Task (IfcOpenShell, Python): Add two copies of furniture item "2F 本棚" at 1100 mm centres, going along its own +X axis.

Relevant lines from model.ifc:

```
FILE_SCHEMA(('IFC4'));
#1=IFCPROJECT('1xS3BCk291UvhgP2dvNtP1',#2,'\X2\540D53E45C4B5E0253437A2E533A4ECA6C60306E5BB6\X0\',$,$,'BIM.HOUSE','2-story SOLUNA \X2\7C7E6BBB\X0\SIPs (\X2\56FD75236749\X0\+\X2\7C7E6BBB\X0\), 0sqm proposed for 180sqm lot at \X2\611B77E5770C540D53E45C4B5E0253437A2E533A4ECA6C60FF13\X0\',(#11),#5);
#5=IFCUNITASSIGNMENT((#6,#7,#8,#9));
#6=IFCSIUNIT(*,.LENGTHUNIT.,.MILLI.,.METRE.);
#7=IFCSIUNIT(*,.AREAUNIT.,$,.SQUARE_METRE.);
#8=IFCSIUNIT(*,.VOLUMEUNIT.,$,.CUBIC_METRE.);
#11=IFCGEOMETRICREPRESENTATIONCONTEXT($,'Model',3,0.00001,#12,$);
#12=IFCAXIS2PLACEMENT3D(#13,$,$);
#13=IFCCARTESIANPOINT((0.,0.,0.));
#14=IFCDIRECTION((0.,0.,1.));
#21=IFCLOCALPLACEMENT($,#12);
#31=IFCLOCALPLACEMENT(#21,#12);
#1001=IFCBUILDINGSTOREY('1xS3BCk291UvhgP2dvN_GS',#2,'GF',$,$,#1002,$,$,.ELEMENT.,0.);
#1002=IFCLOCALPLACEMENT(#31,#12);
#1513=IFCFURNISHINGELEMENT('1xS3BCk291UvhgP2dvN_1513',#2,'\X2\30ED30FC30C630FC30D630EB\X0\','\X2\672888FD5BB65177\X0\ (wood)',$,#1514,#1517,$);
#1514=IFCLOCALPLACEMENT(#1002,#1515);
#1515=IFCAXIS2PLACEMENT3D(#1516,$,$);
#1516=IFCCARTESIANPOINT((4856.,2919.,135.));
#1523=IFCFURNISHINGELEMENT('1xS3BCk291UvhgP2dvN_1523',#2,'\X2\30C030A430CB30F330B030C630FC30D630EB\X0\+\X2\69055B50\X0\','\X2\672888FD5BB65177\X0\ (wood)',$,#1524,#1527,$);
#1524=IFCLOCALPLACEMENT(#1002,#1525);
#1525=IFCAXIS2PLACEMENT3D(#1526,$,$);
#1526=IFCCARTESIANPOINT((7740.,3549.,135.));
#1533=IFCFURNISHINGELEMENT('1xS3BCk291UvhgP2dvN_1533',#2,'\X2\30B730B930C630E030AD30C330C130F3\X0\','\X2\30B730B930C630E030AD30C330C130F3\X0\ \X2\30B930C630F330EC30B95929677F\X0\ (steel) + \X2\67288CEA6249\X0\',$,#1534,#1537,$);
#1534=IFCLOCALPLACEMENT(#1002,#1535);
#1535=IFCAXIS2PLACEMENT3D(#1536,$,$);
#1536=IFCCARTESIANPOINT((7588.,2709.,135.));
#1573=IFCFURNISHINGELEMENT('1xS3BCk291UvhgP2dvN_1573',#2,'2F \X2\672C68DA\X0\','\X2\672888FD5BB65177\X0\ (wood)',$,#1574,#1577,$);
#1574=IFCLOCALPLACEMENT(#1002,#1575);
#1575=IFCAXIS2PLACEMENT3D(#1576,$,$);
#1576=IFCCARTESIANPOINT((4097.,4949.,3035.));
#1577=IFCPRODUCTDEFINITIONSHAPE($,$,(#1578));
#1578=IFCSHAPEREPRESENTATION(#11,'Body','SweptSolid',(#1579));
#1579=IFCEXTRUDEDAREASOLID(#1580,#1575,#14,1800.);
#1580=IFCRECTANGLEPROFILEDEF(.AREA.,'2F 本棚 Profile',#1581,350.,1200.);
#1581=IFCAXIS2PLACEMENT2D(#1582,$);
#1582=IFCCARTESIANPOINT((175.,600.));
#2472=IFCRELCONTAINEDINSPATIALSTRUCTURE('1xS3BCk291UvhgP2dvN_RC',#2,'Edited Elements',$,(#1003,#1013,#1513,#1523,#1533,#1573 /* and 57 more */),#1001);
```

```python
import ifcopenshell
import ifcopenshell.api.geometry
import ifcopenshell.api.root
import ifcopenshell.util.element
import ifcopenshell.util.placement

model = ifcopenshell.open("model.ifc")


def reuse_history(source, copy):
    """copy_class also copies each property set's owner history, people and application; keep the originals."""
    for rel in copy.IsDefinedBy:
        if rel.is_a("IfcRelDefinesByProperties") and (history := rel.RelatingPropertyDefinition.OwnerHistory):
            rel.RelatingPropertyDefinition.OwnerHistory = source.OwnerHistory
            ifcopenshell.util.element.remove_deep2(model, history)


source = model.by_guid("1xS3BCk291UvhgP2dvN_1573")
base = ifcopenshell.util.placement.get_local_placement(source.ObjectPlacement)
step = base[:3, 0] * 1100.0

for i in range(1, 3):
    copy = ifcopenshell.api.root.copy_class(model, product=source)
    copy.Representation = ifcopenshell.util.element.copy_deep(
        model, source.Representation, exclude=["IfcGeometricRepresentationContext", "IfcRepresentationMap"]
    )
    reuse_history(source, copy)
    matrix = base.copy()
    matrix[:3, 3] += i * step
    print("added at", matrix[:3, 3].round(3) + 0.0)
    ifcopenshell.api.geometry.edit_object_placement(model, product=copy, matrix=matrix, is_si=False)

model.write("model_rev.ifc")
```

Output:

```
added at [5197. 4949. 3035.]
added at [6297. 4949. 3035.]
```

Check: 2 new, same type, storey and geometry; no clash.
